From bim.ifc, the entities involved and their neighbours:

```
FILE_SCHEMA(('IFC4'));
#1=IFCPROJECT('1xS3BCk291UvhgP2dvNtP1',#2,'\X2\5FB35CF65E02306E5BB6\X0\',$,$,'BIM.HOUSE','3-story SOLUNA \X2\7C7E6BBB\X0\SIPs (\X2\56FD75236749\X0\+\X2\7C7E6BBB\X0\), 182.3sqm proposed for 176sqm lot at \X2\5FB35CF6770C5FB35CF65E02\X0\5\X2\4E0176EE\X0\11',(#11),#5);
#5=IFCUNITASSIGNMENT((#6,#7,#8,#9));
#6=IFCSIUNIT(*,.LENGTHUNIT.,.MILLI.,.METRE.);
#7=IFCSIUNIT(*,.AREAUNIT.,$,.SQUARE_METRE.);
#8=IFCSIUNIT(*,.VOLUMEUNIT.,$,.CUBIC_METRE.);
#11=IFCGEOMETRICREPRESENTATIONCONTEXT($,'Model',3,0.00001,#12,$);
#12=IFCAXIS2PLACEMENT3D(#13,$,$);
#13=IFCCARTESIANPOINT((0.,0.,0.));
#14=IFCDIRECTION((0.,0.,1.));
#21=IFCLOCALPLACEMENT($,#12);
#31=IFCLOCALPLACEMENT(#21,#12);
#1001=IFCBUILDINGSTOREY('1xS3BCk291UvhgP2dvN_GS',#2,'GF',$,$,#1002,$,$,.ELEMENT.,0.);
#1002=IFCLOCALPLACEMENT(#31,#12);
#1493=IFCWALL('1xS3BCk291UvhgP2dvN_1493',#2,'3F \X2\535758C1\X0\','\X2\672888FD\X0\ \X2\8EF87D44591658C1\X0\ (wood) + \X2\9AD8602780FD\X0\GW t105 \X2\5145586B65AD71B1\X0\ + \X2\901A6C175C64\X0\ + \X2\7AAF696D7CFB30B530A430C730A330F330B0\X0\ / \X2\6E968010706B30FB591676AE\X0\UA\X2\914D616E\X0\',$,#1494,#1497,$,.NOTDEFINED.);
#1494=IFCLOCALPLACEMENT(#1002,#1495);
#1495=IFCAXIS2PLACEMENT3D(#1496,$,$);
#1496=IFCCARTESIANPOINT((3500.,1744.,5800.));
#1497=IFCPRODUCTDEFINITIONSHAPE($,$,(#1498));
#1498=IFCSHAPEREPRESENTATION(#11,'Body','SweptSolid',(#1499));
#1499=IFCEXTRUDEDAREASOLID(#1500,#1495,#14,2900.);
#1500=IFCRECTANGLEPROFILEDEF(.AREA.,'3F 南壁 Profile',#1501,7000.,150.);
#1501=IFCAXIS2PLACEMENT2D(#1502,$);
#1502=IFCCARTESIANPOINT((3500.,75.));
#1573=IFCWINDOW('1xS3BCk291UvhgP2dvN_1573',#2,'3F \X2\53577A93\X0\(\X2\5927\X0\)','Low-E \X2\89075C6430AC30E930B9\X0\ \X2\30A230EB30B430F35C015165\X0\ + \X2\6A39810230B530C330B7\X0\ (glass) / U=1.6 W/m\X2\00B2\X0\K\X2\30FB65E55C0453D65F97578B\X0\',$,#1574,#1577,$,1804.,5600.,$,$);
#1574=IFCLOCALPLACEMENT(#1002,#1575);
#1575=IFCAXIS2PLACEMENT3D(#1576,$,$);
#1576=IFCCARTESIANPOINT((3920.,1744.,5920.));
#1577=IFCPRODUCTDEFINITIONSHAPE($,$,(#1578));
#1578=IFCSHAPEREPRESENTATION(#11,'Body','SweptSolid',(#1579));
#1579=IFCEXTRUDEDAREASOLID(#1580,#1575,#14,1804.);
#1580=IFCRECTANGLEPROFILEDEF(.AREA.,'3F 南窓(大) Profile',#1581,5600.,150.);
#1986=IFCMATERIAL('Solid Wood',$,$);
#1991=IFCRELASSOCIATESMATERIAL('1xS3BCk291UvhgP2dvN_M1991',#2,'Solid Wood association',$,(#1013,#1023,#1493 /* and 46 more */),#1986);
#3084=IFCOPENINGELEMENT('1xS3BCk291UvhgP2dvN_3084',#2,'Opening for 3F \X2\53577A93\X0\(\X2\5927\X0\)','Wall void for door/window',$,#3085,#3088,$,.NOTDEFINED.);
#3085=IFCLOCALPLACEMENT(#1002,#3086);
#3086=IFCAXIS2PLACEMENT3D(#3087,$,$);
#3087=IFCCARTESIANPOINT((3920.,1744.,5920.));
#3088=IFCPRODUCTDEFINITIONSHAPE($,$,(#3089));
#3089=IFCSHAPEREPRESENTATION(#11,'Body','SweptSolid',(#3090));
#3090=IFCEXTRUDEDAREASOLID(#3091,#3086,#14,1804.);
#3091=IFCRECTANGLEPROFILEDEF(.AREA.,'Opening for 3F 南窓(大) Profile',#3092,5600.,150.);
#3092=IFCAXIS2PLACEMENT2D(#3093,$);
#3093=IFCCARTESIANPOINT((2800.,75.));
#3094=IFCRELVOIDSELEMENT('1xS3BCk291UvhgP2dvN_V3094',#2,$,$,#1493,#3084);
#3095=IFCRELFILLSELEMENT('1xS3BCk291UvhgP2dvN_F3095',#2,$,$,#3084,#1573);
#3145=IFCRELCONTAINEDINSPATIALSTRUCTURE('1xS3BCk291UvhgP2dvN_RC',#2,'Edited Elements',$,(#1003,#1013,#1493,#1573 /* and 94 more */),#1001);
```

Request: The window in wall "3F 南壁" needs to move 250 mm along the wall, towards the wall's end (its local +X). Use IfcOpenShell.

```python
import ifcopenshell
import ifcopenshell.api.geometry
import ifcopenshell.util.placement
import ifcopenshell.util.unit

model = ifcopenshell.open("bim.ifc")
unit_scale = ifcopenshell.util.unit.calculate_unit_scale(model)

window = model.by_id(1573)
opening = window.FillsVoids[0].RelatingOpeningElement
wall = opening.VoidsElements[0].RelatingBuildingElement

wall_matrix = ifcopenshell.util.placement.get_local_placement(wall.ObjectPlacement)
shift = wall_matrix[:3, 0] * 0.25 / unit_scale
before = ifcopenshell.util.placement.get_local_placement(window.ObjectPlacement)[:3, 3].copy()

# The window is not placed relative to its opening, so move both.
for product in (opening, window):
    matrix = ifcopenshell.util.placement.get_local_placement(product.ObjectPlacement)
    matrix[:3, 3] += shift
    ifcopenshell.api.geometry.edit_object_placement(model, product=product, matrix=matrix, is_si=False)

after = ifcopenshell.util.placement.get_local_placement(window.ObjectPlacement)[:3, 3]
print("window moved by", (after - before).round(3) + 0.0)

model.write("bim-out.ifc")
```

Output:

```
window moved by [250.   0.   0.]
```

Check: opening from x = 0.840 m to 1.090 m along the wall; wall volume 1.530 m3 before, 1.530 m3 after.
